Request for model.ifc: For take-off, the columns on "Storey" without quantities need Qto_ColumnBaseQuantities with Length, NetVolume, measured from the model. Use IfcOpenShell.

First a look at what the model holds.

```python
import ifcopenshell
import ifcopenshell.util.element
import ifcopenshell.util.unit

model = ifcopenshell.open("model.ifc")
print(model.schema)
for unit_type in ("LENGTHUNIT", "AREAUNIT", "VOLUMEUNIT"):
    print(unit_type, ifcopenshell.util.unit.calculate_unit_scale(model, unit_type))
storey = next(s for s in model.by_type("IfcBuildingStorey") if s.Name == "Storey")
columns = [e for e in ifcopenshell.util.element.get_decomposition(storey) if e.is_a("IfcColumn")]
for e in sorted(columns, key=lambda e: e.id()):
    print(e.id(), e.is_a(), e.Name, list(ifcopenshell.util.element.get_psets(e, qtos_only=True)), sep=" | ")
```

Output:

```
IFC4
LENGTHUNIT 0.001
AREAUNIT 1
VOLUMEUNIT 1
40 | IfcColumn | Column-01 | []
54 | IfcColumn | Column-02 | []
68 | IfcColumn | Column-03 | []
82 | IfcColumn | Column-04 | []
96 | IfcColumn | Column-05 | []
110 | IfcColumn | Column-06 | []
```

```python
import ifcopenshell
import ifcopenshell.api.pset
import ifcopenshell.geom
import ifcopenshell.util.element
import ifcopenshell.util.shape
import ifcopenshell.util.unit

model = ifcopenshell.open("model.ifc")
unit_scale = ifcopenshell.util.unit.calculate_unit_scale(model)
volume_scale = ifcopenshell.util.unit.calculate_unit_scale(model, "VOLUMEUNIT")
settings = ifcopenshell.geom.settings()

storey = next(s for s in model.by_type("IfcBuildingStorey") if s.Name == "Storey")
columns = [e for e in ifcopenshell.util.element.get_decomposition(storey) if e.is_a("IfcColumn")]

for e in sorted(columns, key=lambda e: e.id()):
    if ifcopenshell.util.element.get_psets(e, qtos_only=True, should_inherit=False):
        continue
    # Geometry comes back in metres, in the element's own axes.
    shape = ifcopenshell.geom.create_shape(settings, e)
    values = {
        "Length": ifcopenshell.util.shape.get_z(shape.geometry) / unit_scale,
        "NetVolume": ifcopenshell.util.shape.get_volume(shape.geometry) / volume_scale,
    }
    qto = ifcopenshell.api.pset.add_qto(model, product=e, name="Qto_ColumnBaseQuantities")
    ifcopenshell.api.pset.edit_qto(model, qto=qto, properties=values)
    print(e.id(), {k: round(v, 3) for k, v in values.items()})

model.write("model-out.ifc")
```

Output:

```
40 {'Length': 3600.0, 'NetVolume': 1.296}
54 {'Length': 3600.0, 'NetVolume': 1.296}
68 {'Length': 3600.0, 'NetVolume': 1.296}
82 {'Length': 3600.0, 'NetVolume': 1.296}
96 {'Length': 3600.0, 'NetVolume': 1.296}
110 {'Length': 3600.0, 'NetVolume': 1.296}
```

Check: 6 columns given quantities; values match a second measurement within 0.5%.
